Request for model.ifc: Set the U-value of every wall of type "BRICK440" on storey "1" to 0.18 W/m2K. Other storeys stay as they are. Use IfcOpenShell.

First a look at what the model holds.

```python
import ifcopenshell
import ifcopenshell.util.element

model = ifcopenshell.open("model.ifc")
print(model.schema)
storey = next(s for s in model.by_type("IfcBuildingStorey") if s.Name == "1")
walls = [e for e in ifcopenshell.util.element.get_decomposition(storey) if e.is_a("IfcWall")]
seen = {}
for e in walls:
    element_type = ifcopenshell.util.element.get_type(e)
    key = (element_type.Name if element_type != e and element_type else None, ifcopenshell.util.element.get_pset(e, "Pset_WallCommon", "ThermalTransmittance"))
    seen[key] = seen.get(key, 0) + 1
for (name, value), count in sorted(seen.items(), key=str):
    print(count, "x", name, "|", value)
```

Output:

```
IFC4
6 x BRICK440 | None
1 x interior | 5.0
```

```python
import ifcopenshell
import ifcopenshell.api.pset
import ifcopenshell.util.element

model = ifcopenshell.open("model.ifc")

storey = next(s for s in model.by_type("IfcBuildingStorey") if s.Name == "1")
walls = [e for e in ifcopenshell.util.element.get_decomposition(storey) if e.is_a("IfcWall")]

count = 0
for e in walls:
    element_type = ifcopenshell.util.element.get_type(e)
    if element_type in (None, e) or element_type.Name != "BRICK440":
        continue
    # add_pset returns the element's existing set when there is one.
    pset = ifcopenshell.api.pset.add_pset(model, product=e, name="Pset_WallCommon")
    ifcopenshell.api.pset.edit_pset(model, pset=pset, properties={"ThermalTransmittance": 0.18})
    count += 1

print(count, "walls updated")

model.write("model_updated.ifc")
```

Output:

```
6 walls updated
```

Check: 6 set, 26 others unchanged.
